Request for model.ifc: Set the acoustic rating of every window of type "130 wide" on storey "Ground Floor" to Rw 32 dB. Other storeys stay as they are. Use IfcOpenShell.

First a look at what the model holds.

```python
import ifcopenshell
import ifcopenshell.util.element

model = ifcopenshell.open("model.ifc")
print(model.schema)
storey = next(s for s in model.by_type("IfcBuildingStorey") if s.Name == "Ground Floor")
windows = [e for e in ifcopenshell.util.element.get_decomposition(storey) if e.is_a("IfcWindow")]
seen = {}
for e in windows:
    element_type = ifcopenshell.util.element.get_type(e)
    key = (element_type.Name if element_type != e and element_type else None, ifcopenshell.util.element.get_pset(e, "Pset_WindowCommon", "AcousticRating"))
    seen[key] = seen.get(key, 0) + 1
for (name, value), count in sorted(seen.items(), key=str):
    print(count, "x", name, "|", value)
```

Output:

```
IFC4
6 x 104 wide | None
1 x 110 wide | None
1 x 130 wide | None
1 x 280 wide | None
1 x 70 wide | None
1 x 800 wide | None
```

```python
import ifcopenshell
import ifcopenshell.api.pset
import ifcopenshell.util.element

model = ifcopenshell.open("model.ifc")

storey = next(s for s in model.by_type("IfcBuildingStorey") if s.Name == "Ground Floor")
windows = [e for e in ifcopenshell.util.element.get_decomposition(storey) if e.is_a("IfcWindow")]

count = 0
for e in windows:
    element_type = ifcopenshell.util.element.get_type(e)
    if element_type in (None, e) or element_type.Name != "130 wide":
        continue
    # add_pset returns the element's existing set when there is one.
    pset = ifcopenshell.api.pset.add_pset(model, product=e, name="Pset_WindowCommon")
    ifcopenshell.api.pset.edit_pset(model, pset=pset, properties={"AcousticRating": "Rw 32 dB"})
    count += 1

print(count, "windows updated")

model.write("model-out.ifc")
```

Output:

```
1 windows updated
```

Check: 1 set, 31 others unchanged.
